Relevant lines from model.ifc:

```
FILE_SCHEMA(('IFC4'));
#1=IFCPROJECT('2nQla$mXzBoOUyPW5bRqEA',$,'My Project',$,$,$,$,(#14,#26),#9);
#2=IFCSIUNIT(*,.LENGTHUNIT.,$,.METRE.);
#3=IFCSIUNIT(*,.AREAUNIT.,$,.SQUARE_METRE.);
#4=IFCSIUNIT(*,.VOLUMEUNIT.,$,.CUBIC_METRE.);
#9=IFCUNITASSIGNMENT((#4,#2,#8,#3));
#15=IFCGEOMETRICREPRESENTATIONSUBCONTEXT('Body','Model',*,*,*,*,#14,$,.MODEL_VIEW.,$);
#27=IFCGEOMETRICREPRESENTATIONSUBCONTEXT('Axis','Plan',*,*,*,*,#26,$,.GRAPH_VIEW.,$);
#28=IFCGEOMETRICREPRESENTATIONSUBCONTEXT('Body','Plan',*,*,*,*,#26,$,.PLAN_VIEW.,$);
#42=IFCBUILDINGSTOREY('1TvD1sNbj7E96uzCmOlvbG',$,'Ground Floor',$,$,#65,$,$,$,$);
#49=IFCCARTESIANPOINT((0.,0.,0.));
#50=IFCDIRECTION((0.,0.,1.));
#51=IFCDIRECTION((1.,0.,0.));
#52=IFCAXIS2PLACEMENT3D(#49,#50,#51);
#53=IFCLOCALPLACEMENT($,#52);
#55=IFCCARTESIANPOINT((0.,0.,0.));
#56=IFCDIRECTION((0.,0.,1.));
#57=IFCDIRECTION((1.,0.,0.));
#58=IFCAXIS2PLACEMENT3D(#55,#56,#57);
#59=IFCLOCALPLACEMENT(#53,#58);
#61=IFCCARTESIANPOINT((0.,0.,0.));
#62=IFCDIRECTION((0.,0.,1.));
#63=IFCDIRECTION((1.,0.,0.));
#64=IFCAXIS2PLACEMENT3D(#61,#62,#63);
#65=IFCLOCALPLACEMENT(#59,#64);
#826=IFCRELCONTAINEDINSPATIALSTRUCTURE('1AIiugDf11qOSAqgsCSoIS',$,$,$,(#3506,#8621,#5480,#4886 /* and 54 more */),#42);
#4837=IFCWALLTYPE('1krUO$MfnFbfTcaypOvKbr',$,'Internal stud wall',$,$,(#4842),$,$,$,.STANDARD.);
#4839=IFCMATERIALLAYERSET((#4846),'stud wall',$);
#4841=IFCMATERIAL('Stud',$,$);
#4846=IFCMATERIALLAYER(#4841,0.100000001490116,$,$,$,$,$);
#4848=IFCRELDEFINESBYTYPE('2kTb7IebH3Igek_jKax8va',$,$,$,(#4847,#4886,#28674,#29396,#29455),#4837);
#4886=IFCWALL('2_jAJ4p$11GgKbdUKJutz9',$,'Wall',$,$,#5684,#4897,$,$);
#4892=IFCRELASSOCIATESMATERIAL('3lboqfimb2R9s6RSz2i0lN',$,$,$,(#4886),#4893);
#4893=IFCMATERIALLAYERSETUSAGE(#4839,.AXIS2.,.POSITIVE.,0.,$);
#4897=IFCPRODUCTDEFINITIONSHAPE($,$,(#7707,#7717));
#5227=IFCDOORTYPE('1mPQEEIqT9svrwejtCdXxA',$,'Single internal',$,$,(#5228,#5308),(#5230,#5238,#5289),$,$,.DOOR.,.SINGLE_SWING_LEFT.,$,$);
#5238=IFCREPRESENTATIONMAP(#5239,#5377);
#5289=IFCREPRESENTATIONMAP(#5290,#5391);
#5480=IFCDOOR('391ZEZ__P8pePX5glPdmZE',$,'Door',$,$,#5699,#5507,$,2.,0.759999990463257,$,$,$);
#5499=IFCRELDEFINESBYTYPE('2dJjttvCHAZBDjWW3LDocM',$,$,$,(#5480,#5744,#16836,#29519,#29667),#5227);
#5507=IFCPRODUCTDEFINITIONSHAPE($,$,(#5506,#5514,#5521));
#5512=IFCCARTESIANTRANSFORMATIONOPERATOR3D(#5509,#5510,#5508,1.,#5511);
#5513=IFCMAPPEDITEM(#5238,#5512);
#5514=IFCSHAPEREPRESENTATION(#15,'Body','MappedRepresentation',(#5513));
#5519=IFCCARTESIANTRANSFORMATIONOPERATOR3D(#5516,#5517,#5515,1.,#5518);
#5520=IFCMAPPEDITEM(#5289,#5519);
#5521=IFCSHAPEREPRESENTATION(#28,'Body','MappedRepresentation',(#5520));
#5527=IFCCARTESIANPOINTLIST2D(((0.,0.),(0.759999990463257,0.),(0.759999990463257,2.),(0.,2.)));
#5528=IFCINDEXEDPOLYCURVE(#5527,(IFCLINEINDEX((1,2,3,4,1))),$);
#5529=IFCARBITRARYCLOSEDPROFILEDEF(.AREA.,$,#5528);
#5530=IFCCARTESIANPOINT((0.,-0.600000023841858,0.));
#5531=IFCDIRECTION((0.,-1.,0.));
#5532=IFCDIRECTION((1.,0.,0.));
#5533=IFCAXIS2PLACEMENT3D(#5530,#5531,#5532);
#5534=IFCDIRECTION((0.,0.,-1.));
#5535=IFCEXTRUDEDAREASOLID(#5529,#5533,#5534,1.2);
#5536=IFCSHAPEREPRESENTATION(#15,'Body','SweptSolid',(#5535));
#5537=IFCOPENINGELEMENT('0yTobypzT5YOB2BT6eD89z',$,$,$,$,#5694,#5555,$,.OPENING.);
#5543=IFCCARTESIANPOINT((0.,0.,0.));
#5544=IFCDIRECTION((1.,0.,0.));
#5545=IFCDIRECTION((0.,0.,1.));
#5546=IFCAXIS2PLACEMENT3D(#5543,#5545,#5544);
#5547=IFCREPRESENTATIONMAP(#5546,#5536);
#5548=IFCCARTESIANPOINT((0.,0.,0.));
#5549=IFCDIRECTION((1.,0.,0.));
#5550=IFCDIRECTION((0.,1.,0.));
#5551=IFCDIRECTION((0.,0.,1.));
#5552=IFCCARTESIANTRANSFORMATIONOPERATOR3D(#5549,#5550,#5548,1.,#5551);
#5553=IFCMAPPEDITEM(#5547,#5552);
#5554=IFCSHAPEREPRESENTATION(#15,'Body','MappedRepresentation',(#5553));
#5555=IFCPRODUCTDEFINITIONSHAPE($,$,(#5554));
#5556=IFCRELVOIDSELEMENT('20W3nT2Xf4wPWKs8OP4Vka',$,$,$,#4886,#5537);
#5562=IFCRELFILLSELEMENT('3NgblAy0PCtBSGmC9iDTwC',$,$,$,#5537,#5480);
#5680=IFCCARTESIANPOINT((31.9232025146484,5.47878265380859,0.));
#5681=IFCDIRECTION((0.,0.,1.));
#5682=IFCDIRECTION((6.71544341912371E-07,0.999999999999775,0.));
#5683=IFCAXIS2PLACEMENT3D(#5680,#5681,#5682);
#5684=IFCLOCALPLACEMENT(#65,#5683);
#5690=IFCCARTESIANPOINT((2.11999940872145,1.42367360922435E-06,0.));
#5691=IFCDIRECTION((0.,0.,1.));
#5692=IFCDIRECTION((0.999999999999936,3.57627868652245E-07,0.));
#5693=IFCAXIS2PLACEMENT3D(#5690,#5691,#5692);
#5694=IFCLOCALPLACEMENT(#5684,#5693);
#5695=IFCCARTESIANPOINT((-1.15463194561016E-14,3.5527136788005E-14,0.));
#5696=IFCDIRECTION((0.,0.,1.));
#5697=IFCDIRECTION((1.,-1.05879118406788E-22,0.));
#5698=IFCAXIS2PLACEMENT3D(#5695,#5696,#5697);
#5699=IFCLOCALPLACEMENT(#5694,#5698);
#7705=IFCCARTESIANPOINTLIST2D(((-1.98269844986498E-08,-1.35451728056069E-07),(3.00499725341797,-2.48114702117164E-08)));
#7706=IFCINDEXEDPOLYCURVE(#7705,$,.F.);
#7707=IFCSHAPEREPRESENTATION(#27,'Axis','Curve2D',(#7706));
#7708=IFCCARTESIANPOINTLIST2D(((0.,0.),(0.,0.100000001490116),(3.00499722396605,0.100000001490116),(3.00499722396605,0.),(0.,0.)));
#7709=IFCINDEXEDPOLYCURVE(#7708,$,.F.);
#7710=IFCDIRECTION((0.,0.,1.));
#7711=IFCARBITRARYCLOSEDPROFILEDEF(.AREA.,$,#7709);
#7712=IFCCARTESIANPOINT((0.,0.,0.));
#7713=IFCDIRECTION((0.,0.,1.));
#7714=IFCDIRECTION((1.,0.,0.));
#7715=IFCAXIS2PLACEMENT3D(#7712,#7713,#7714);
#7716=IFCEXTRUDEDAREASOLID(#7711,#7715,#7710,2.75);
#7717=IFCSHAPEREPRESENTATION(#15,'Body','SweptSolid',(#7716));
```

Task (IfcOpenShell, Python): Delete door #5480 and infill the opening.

```python
import ifcopenshell
import ifcopenshell.api.feature
import ifcopenshell.api.root
import ifcopenshell.geom
import ifcopenshell.util.shape

model = ifcopenshell.open("model.ifc")
settings = ifcopenshell.geom.settings()


def volume(element):
    """Net volume in cubic metres, openings subtracted."""
    shape = ifcopenshell.geom.create_shape(settings, element)
    return ifcopenshell.util.shape.get_volume(shape.geometry)


door = model.by_guid("391ZEZ__P8pePX5glPdmZE")
opening = door.FillsVoids[0].RelatingOpeningElement
wall = opening.VoidsElements[0].RelatingBuildingElement
before = volume(wall)

ifcopenshell.api.root.remove_product(model, product=door)
ifcopenshell.api.feature.remove_feature(model, feature=opening)

after = volume(wall)

print(f"wall volume {before:.3f} -> {after:.3f} m3")

model.write("model_rev.ifc")
```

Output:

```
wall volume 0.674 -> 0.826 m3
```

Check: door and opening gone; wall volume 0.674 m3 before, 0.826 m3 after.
